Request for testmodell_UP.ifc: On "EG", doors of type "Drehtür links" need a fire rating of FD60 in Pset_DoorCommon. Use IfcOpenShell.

First a look at what the model holds.

```python
import ifcopenshell
import ifcopenshell.util.element

model = ifcopenshell.open("testmodell_UP.ifc")
print(model.schema)
storey = next(s for s in model.by_type("IfcBuildingStorey") if s.Name == "EG")
doors = [e for e in ifcopenshell.util.element.get_decomposition(storey) if e.is_a("IfcDoor")]
seen = {}
for e in doors:
    element_type = ifcopenshell.util.element.get_type(e)
    key = (element_type.Name if element_type != e and element_type else None, ifcopenshell.util.element.get_pset(e, "Pset_DoorCommon", "FireRating"))
    seen[key] = seen.get(key, 0) + 1
for (name, value), count in sorted(seen.items(), key=str):
    print(count, "x", name, "|", value)
```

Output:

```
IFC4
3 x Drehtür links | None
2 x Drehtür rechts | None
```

```python
import ifcopenshell
import ifcopenshell.api.pset
import ifcopenshell.util.element

model = ifcopenshell.open("testmodell_UP.ifc")

storey = next(s for s in model.by_type("IfcBuildingStorey") if s.Name == "EG")
doors = [e for e in ifcopenshell.util.element.get_decomposition(storey) if e.is_a("IfcDoor")]

count = 0
for e in doors:
    element_type = ifcopenshell.util.element.get_type(e)
    if element_type in (None, e) or element_type.Name != "Drehtür links":
        continue
    # add_pset returns the element's existing set when there is one.
    pset = ifcopenshell.api.pset.add_pset(model, product=e, name="Pset_DoorCommon")
    ifcopenshell.api.pset.edit_pset(model, pset=pset, properties={"FireRating": "FD60"})
    count += 1

print(count, "doors updated")

model.write("testmodell_UP_rev.ifc")
```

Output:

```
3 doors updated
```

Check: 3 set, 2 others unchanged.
